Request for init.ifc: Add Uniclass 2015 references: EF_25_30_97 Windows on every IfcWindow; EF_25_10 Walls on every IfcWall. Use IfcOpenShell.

First a look at what the model holds.

```python
import ifcopenshell

model = ifcopenshell.open("init.ifc")
print(model.schema)
print("classifications:", [c.Name for c in model.by_type("IfcClassification")])
for ifc_class in ("IfcDoor", "IfcRoof", "IfcStair", "IfcWall", "IfcWindow"):
    print(ifc_class, len(model.by_type(ifc_class)))
```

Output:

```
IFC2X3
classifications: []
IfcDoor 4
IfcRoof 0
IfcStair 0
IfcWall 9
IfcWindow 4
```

```python
import ifcopenshell
import ifcopenshell.api.classification

model = ifcopenshell.open("init.ifc")

# IFC2X3 requires Source and Edition and has no link from the project to the system.
system = model.create_entity("IfcClassification", Source="NBS", Edition="2015", Name="Uniclass 2015")

codes = {
    "IfcWindow": ("EF_25_30_97", "Windows"),
    "IfcWall": ("EF_25_10", "Walls"),
}
for ifc_class, (code, name) in codes.items():
    products = model.by_type(ifc_class)
    ifcopenshell.api.classification.add_reference(
        model, products=products, classification=system, identification=code, name=name
    )
    print(code, len(products))

model.write("init_rev.ifc")
```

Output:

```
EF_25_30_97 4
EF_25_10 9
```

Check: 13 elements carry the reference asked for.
